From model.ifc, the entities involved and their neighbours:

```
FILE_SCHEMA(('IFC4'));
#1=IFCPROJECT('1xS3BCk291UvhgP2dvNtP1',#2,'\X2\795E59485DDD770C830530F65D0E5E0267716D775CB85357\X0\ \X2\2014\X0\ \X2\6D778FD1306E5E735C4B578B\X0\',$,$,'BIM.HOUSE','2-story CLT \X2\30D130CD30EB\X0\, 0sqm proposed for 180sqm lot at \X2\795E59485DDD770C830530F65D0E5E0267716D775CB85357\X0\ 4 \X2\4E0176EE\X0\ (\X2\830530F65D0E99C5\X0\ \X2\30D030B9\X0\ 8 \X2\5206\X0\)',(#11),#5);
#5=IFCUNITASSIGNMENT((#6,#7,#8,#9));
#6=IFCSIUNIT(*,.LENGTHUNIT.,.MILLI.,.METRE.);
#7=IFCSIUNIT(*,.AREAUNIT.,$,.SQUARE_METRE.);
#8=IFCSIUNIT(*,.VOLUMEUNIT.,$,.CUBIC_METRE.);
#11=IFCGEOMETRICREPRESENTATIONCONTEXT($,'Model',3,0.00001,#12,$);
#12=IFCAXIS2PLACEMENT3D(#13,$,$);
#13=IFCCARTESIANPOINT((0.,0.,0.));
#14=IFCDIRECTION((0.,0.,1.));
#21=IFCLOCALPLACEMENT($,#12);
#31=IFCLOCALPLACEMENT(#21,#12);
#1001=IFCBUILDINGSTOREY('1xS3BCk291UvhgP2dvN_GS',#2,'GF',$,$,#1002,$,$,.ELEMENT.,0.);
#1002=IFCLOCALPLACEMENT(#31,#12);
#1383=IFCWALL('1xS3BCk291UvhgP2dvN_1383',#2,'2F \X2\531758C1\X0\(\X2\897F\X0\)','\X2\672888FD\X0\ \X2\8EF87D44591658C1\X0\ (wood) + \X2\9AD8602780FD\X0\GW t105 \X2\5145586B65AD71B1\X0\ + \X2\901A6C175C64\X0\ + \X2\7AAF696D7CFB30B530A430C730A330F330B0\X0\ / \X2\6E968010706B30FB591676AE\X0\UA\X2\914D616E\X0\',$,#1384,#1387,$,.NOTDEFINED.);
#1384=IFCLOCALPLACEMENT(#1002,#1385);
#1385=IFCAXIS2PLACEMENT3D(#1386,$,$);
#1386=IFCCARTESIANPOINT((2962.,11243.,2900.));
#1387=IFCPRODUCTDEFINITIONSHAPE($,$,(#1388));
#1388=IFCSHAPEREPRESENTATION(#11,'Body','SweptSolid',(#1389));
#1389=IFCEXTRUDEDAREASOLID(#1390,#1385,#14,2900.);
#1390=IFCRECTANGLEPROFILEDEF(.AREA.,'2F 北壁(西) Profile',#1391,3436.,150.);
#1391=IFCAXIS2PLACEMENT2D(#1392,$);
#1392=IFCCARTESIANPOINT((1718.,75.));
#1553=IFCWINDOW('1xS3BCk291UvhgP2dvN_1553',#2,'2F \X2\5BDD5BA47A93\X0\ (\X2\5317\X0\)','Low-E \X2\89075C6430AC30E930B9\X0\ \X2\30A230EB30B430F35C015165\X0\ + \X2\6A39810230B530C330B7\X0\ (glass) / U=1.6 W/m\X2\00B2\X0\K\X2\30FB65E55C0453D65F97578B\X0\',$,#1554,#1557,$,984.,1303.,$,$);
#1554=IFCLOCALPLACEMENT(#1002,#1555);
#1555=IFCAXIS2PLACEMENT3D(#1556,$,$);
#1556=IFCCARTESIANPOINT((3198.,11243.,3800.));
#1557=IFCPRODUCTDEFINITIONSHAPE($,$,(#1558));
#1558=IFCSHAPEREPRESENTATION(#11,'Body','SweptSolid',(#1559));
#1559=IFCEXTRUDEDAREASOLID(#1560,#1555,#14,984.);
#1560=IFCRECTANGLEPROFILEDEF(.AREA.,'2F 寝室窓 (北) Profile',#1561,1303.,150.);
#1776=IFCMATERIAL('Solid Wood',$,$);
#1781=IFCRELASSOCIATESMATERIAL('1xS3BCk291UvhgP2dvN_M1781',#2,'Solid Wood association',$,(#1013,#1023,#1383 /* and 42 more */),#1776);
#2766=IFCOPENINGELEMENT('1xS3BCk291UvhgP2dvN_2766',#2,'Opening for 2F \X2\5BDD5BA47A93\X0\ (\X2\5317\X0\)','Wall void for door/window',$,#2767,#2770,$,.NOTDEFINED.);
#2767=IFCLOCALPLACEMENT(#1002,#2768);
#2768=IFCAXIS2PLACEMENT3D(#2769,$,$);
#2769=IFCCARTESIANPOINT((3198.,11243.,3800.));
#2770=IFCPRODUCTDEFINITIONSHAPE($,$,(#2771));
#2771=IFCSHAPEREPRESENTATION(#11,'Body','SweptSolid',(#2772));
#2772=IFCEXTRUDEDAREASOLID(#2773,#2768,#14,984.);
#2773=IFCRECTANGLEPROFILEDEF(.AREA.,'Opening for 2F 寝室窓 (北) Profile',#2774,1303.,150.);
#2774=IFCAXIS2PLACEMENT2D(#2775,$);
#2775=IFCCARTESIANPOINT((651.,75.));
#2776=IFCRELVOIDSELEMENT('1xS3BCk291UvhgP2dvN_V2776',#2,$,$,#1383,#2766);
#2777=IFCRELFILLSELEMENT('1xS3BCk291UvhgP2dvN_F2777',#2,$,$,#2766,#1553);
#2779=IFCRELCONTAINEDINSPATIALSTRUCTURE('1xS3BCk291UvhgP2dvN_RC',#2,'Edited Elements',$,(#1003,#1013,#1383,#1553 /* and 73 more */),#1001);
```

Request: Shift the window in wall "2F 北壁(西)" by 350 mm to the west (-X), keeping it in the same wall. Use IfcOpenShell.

```python
import ifcopenshell
import ifcopenshell.api.geometry
import ifcopenshell.util.placement
import ifcopenshell.util.unit

model = ifcopenshell.open("model.ifc")
unit_scale = ifcopenshell.util.unit.calculate_unit_scale(model)

window = model.by_guid("1xS3BCk291UvhgP2dvN_1553")
opening = window.FillsVoids[0].RelatingOpeningElement
wall = opening.VoidsElements[0].RelatingBuildingElement

wall_matrix = ifcopenshell.util.placement.get_local_placement(wall.ObjectPlacement)
shift = wall_matrix[:3, 0] * -0.35 / unit_scale
before = ifcopenshell.util.placement.get_local_placement(window.ObjectPlacement)[:3, 3].copy()

# The window is not placed relative to its opening, so move both.
for product in (opening, window):
    matrix = ifcopenshell.util.placement.get_local_placement(product.ObjectPlacement)
    matrix[:3, 3] += shift
    ifcopenshell.api.geometry.edit_object_placement(model, product=product, matrix=matrix, is_si=False)

after = ifcopenshell.util.placement.get_local_placement(window.ObjectPlacement)[:3, 3]
print("window moved by", (after - before).round(3) + 0.0)

model.write("model_edited.ifc")
```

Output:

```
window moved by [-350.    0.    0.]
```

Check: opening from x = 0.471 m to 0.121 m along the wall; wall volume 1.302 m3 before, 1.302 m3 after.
